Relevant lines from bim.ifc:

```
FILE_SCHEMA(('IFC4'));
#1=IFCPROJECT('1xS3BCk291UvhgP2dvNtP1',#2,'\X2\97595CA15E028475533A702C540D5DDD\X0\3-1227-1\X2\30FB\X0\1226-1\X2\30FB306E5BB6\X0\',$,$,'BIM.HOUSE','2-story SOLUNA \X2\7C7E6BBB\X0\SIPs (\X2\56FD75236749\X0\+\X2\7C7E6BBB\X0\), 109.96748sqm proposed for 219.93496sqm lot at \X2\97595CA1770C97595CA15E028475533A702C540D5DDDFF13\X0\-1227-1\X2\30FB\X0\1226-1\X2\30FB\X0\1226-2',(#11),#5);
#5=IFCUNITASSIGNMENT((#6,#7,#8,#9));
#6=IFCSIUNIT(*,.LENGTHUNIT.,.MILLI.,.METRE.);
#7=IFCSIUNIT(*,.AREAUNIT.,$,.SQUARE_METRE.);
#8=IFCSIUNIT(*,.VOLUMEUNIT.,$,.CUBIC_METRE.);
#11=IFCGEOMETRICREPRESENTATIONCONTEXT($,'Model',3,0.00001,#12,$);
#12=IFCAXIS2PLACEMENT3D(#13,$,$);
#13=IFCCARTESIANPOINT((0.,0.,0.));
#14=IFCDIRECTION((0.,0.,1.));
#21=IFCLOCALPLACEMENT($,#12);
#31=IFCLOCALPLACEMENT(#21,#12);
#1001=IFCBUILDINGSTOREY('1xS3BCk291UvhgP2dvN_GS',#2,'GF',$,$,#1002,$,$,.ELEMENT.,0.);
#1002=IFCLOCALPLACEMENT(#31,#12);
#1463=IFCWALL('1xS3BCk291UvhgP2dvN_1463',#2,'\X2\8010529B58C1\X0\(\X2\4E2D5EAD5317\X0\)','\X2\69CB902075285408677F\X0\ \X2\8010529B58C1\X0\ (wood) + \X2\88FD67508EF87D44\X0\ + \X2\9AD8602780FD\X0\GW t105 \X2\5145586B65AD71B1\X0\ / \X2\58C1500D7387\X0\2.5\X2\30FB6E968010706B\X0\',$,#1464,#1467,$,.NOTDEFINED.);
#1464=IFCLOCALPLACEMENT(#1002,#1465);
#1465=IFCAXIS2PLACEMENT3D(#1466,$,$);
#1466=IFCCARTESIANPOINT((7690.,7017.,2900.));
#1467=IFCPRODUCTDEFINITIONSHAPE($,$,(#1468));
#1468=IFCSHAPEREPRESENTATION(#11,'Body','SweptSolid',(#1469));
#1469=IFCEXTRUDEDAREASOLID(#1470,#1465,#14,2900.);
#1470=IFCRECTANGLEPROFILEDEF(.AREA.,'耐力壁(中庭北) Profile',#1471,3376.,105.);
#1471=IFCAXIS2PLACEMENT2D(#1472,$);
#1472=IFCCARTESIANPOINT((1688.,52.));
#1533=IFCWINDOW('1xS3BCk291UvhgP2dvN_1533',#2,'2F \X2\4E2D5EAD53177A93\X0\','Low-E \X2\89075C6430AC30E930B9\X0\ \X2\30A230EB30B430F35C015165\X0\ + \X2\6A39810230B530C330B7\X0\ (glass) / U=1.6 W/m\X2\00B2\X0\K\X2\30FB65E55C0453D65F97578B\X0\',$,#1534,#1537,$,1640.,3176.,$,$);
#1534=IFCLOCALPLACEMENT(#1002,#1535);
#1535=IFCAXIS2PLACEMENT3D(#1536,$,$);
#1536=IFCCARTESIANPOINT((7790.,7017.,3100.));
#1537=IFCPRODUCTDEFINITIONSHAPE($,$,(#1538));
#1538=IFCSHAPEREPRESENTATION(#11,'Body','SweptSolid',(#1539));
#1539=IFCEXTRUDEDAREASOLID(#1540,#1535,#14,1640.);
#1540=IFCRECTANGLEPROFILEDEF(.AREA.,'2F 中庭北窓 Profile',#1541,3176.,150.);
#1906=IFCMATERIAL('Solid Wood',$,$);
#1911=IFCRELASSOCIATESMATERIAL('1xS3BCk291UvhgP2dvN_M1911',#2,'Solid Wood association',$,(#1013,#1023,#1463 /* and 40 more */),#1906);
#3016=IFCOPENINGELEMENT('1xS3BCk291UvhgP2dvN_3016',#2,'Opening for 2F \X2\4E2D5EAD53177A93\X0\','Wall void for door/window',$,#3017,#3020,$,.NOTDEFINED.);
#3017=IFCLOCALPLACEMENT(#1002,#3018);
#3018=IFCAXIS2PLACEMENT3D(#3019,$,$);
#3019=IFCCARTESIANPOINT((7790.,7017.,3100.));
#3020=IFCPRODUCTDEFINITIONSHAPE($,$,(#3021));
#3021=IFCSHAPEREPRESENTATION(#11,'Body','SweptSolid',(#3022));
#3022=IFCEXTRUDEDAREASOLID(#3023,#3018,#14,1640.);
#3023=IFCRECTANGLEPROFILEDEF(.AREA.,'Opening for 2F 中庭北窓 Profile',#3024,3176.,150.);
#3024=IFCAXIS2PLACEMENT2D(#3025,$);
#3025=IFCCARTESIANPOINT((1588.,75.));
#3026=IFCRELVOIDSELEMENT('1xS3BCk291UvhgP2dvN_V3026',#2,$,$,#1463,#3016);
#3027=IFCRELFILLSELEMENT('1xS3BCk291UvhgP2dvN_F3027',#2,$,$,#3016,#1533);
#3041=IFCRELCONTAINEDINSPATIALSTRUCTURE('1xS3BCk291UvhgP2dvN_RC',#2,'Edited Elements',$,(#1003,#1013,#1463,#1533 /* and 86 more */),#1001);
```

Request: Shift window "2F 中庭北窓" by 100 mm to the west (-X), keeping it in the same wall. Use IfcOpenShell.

```python
import ifcopenshell
import ifcopenshell.api.geometry
import ifcopenshell.util.placement

model = ifcopenshell.open("bim.ifc")

window = model.by_guid("1xS3BCk291UvhgP2dvN_1533")
opening = window.FillsVoids[0].RelatingOpeningElement
wall = opening.VoidsElements[0].RelatingBuildingElement

wall_matrix = ifcopenshell.util.placement.get_local_placement(wall.ObjectPlacement)
shift = wall_matrix[:3, 0] * -100.0
before = ifcopenshell.util.placement.get_local_placement(window.ObjectPlacement)[:3, 3].copy()

# The window is not placed relative to its opening, so move both.
for product in (opening, window):
    matrix = ifcopenshell.util.placement.get_local_placement(product.ObjectPlacement)
    matrix[:3, 3] += shift
    ifcopenshell.api.geometry.edit_object_placement(model, product=product, matrix=matrix, is_si=False)

after = ifcopenshell.util.placement.get_local_placement(window.ObjectPlacement)[:3, 3]
print("window moved by", (after - before).round(3) + 0.0)

model.write("bim_edited.ifc")
```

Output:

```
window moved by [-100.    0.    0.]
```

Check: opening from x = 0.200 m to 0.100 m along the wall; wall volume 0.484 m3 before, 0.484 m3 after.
